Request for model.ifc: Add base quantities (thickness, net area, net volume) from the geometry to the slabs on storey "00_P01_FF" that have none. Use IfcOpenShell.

First a look at what the model holds.

```python
import ifcopenshell
import ifcopenshell.util.element
import ifcopenshell.util.unit

model = ifcopenshell.open("model.ifc")
print(model.schema)
for unit_type in ("LENGTHUNIT", "AREAUNIT", "VOLUMEUNIT"):
    print(unit_type, ifcopenshell.util.unit.calculate_unit_scale(model, unit_type))
storey = next(s for s in model.by_type("IfcBuildingStorey") if s.Name == "00_P01_FF")
slabs = [e for e in ifcopenshell.util.element.get_decomposition(storey) if e.is_a("IfcSlab")]
for e in sorted(slabs, key=lambda e: e.id()):
    print(e.id(), e.is_a(), e.Name, list(ifcopenshell.util.element.get_psets(e, qtos_only=True)), sep=" | ")
```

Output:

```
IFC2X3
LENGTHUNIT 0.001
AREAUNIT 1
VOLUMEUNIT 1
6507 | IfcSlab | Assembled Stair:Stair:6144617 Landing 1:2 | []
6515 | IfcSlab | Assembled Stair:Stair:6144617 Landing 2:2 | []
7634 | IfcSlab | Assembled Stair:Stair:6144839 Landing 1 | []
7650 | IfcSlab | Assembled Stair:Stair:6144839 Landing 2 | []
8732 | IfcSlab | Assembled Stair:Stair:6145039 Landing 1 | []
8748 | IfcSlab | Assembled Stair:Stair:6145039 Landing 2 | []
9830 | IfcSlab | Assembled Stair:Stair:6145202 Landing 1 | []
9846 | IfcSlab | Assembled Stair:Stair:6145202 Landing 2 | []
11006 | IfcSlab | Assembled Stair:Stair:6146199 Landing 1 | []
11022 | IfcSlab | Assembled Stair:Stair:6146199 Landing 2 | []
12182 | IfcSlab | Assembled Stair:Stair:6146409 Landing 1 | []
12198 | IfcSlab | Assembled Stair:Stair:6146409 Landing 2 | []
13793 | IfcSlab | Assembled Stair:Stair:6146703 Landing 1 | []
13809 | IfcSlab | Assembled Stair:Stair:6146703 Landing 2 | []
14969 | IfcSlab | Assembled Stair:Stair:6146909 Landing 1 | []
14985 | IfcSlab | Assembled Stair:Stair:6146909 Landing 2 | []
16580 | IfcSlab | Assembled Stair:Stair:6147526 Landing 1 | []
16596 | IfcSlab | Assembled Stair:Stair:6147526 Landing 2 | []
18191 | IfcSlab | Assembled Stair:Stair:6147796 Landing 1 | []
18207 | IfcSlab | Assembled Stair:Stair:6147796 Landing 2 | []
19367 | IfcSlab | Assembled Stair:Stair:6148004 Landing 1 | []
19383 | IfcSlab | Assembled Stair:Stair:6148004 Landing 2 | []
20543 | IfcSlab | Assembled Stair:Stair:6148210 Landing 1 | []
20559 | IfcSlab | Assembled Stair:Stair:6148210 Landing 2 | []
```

```python
import ifcopenshell
import ifcopenshell.api.pset
import ifcopenshell.geom
import ifcopenshell.util.element
import ifcopenshell.util.shape
import ifcopenshell.util.unit

model = ifcopenshell.open("model.ifc")
unit_scale = ifcopenshell.util.unit.calculate_unit_scale(model)
area_scale = ifcopenshell.util.unit.calculate_unit_scale(model, "AREAUNIT")
volume_scale = ifcopenshell.util.unit.calculate_unit_scale(model, "VOLUMEUNIT")
settings = ifcopenshell.geom.settings()

storey = next(s for s in model.by_type("IfcBuildingStorey") if s.Name == "00_P01_FF")
slabs = [e for e in ifcopenshell.util.element.get_decomposition(storey) if e.is_a("IfcSlab")]

for e in sorted(slabs, key=lambda e: e.id()):
    if ifcopenshell.util.element.get_psets(e, qtos_only=True, should_inherit=False):
        continue
    # Geometry comes back in metres, in the element's own axes.
    shape = ifcopenshell.geom.create_shape(settings, e)
    values = {
        "Width": ifcopenshell.util.shape.get_z(shape.geometry) / unit_scale,
        "NetArea": ifcopenshell.util.shape.get_footprint_area(shape.geometry) / area_scale,
        "NetVolume": ifcopenshell.util.shape.get_volume(shape.geometry) / volume_scale,
    }
    qto = ifcopenshell.api.pset.add_qto(model, product=e, name="BaseQuantities")
    ifcopenshell.api.pset.edit_qto(model, qto=qto, properties=values)
    print(e.id(), {k: round(v, 3) for k, v in values.items()})

model.write("model_edited.ifc")
```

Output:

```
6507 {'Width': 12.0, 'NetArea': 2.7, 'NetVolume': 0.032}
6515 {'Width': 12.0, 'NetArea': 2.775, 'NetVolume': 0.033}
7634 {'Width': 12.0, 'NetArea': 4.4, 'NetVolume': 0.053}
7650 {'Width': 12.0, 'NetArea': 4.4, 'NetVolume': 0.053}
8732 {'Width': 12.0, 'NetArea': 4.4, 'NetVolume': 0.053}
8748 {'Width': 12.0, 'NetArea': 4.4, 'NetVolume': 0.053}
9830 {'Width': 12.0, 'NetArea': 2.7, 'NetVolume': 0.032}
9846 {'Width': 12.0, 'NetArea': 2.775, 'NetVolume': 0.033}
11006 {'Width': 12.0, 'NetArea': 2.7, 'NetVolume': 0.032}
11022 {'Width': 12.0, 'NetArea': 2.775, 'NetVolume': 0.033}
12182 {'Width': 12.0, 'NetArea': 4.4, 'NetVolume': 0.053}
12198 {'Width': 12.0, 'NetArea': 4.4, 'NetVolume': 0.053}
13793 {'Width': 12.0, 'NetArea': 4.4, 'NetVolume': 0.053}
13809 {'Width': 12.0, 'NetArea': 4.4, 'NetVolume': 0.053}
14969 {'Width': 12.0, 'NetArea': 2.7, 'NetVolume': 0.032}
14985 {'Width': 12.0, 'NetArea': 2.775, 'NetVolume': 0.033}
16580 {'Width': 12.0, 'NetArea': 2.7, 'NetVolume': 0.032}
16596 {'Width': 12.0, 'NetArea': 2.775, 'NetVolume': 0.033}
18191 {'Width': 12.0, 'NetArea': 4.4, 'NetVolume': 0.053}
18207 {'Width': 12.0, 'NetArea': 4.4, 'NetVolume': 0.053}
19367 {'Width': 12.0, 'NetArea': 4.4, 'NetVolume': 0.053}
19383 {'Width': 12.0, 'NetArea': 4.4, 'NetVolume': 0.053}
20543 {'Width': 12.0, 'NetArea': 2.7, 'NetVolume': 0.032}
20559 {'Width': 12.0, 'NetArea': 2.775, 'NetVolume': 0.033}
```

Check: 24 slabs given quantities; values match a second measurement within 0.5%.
